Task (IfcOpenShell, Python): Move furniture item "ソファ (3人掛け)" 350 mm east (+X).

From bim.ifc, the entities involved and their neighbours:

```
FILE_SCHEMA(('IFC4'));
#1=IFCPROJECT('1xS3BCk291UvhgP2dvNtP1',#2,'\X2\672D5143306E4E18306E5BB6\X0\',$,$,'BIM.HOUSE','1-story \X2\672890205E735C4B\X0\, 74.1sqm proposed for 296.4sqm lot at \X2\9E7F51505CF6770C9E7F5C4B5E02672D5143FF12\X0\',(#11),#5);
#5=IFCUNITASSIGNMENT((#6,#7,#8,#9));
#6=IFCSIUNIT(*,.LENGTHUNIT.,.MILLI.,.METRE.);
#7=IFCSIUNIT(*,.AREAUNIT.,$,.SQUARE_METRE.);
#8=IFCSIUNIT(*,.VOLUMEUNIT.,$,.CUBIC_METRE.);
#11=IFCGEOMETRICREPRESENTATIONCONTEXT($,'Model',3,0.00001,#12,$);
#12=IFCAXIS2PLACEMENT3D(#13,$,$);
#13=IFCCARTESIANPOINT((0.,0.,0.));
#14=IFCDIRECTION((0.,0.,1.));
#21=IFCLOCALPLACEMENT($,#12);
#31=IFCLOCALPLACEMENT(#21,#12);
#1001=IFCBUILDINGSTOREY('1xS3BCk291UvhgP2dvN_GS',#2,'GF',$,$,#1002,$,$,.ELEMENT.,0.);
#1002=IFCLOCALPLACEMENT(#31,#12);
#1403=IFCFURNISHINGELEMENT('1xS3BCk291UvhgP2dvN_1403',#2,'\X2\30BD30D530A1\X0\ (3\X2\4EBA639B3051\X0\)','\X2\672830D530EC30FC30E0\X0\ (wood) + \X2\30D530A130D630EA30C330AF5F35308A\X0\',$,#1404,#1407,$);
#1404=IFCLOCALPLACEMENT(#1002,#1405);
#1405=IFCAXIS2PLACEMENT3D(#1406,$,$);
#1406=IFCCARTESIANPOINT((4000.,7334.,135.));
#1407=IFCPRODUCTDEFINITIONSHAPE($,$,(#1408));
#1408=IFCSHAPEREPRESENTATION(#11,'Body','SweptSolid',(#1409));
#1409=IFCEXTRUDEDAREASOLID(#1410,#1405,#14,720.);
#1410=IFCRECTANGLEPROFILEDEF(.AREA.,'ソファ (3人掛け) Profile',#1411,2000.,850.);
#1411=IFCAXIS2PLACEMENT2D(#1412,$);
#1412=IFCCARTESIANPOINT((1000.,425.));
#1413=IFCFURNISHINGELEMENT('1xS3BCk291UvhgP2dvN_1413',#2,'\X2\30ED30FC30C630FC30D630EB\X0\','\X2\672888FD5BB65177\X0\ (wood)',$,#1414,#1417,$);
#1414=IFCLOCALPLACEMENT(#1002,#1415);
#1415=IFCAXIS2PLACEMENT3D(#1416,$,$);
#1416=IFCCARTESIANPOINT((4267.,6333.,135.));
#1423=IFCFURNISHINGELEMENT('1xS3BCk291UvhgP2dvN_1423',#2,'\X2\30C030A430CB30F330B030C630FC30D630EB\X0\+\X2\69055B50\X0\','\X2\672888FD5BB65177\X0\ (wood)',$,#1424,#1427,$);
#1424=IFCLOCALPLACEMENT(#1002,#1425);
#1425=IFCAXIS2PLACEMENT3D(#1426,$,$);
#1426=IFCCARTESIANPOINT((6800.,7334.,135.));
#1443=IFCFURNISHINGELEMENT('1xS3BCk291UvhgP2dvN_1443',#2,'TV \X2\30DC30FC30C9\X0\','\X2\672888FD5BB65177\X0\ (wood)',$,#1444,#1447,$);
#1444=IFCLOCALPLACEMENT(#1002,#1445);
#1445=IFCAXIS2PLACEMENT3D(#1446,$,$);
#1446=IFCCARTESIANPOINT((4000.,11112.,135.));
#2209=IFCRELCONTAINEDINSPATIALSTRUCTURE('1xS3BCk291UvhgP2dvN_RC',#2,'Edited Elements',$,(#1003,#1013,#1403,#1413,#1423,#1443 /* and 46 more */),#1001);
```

```python
import ifcopenshell
import ifcopenshell.api.geometry
import ifcopenshell.util.placement
import ifcopenshell.util.unit

model = ifcopenshell.open("bim.ifc")
unit_scale = ifcopenshell.util.unit.calculate_unit_scale(model)

item = model.by_guid("1xS3BCk291UvhgP2dvN_1403")
matrix = ifcopenshell.util.placement.get_local_placement(item.ObjectPlacement)
matrix[0, 3] += 0.35 / unit_scale
ifcopenshell.api.geometry.edit_object_placement(model, product=item, matrix=matrix, is_si=False)

print(ifcopenshell.util.placement.get_local_placement(item.ObjectPlacement).round(3) + 0.0)

model.write("bim_rev.ifc")
```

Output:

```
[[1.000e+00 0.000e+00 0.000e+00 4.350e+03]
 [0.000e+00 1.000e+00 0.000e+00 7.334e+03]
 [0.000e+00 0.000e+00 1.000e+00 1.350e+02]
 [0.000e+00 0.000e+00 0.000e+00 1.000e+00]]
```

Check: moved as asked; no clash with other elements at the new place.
